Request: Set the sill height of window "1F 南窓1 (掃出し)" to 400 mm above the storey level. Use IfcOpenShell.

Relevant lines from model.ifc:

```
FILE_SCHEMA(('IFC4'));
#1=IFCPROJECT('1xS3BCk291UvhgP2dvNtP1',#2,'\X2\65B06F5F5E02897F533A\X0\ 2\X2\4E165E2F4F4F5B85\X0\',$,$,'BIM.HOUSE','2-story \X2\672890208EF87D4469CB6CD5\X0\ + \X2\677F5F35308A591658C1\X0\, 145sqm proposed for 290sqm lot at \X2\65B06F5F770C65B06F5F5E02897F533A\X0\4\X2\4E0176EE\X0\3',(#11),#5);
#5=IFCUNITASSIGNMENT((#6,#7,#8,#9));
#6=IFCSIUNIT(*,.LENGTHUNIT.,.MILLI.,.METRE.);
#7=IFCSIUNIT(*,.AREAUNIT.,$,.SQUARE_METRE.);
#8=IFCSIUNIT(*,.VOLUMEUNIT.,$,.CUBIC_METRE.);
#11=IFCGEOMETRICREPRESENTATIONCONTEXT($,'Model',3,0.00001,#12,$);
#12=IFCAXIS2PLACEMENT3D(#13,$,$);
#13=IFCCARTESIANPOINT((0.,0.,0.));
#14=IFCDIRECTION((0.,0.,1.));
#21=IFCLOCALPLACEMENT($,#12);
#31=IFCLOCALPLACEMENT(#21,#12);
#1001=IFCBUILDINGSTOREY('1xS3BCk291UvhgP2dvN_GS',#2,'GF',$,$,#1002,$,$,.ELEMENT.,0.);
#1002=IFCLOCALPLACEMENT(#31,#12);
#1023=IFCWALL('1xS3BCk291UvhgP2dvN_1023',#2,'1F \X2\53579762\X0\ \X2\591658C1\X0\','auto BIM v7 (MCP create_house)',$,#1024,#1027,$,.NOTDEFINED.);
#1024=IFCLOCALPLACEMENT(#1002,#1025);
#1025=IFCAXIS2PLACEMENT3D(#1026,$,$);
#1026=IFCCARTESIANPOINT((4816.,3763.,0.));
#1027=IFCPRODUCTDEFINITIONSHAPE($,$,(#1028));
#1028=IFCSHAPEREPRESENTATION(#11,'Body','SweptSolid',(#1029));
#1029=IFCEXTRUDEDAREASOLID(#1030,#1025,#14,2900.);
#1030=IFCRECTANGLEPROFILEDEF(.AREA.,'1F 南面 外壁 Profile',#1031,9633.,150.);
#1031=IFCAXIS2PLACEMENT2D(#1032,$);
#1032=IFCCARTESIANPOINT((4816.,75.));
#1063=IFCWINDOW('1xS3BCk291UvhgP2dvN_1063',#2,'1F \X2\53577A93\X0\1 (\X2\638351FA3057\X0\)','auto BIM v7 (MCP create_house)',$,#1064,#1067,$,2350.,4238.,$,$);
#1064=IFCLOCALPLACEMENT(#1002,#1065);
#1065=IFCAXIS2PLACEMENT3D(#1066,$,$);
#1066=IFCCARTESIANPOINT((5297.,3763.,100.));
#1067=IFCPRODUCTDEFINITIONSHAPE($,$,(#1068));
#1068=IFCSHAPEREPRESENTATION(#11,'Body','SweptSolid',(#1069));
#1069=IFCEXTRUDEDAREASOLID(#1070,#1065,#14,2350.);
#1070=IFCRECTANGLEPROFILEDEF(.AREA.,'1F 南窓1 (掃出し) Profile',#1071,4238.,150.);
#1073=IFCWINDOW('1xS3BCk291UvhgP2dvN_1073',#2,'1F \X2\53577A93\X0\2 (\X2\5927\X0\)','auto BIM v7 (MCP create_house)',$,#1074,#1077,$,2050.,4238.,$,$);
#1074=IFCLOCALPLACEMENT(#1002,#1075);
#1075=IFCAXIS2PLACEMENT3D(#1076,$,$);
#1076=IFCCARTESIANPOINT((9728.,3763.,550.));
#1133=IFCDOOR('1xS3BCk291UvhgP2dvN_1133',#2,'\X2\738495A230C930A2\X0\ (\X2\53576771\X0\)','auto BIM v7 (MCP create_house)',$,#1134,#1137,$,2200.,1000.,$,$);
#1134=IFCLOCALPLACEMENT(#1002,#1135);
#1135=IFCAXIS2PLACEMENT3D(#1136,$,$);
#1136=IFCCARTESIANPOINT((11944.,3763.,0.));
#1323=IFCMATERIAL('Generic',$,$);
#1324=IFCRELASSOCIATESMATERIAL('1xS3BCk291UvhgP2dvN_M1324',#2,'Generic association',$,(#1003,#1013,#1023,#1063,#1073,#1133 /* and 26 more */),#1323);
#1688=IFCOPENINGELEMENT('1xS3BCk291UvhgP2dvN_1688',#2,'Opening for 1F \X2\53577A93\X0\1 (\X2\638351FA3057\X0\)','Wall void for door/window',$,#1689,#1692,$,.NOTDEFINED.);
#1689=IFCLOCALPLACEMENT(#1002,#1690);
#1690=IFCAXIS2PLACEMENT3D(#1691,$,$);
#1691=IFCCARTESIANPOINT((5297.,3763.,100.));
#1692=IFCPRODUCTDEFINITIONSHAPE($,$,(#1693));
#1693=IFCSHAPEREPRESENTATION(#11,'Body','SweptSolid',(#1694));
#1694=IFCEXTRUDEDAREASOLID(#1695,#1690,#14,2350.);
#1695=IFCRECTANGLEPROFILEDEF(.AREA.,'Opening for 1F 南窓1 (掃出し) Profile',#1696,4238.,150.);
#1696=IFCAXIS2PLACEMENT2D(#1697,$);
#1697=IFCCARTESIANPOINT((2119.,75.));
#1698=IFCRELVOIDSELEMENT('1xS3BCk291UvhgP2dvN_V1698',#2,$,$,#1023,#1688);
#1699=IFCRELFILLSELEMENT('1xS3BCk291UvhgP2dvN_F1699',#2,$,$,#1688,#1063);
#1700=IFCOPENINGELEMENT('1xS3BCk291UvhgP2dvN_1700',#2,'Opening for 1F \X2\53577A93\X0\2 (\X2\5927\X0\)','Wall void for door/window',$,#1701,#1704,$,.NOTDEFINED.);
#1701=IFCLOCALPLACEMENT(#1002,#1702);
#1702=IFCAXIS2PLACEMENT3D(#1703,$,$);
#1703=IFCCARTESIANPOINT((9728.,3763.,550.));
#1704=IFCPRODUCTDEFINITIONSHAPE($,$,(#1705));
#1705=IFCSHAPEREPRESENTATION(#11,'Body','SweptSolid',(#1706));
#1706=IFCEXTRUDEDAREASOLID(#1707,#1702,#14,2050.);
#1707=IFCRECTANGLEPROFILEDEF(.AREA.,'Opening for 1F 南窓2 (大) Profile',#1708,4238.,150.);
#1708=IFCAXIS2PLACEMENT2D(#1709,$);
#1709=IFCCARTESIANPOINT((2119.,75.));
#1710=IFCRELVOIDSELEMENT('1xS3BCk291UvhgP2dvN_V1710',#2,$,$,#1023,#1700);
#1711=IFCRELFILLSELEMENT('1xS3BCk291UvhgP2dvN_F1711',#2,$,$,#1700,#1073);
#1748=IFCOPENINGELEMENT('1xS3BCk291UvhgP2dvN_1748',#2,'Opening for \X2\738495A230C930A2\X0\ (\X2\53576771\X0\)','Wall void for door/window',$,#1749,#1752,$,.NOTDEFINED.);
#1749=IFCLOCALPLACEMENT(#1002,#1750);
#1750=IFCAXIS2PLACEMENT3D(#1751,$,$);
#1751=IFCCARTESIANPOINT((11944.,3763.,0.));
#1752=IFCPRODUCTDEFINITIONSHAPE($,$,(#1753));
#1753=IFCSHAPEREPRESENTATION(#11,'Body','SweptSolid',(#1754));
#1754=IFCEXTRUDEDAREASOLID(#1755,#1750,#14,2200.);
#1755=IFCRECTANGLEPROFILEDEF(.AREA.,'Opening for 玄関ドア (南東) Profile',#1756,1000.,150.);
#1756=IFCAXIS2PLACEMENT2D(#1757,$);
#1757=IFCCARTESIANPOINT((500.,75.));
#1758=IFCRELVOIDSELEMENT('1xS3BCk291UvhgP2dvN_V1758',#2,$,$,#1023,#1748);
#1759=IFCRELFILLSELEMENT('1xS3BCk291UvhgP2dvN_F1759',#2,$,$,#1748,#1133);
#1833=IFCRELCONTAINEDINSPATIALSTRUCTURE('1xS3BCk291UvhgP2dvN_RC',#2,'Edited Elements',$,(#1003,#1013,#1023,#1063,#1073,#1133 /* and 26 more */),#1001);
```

```python
import numpy as np
import ifcopenshell
import ifcopenshell.api.geometry
import ifcopenshell.geom
import ifcopenshell.util.element
import ifcopenshell.util.placement
import ifcopenshell.util.shape
import ifcopenshell.util.unit

model = ifcopenshell.open("model.ifc")
unit_scale = ifcopenshell.util.unit.calculate_unit_scale(model)

window = model.by_guid("1xS3BCk291UvhgP2dvN_1063")
opening = window.FillsVoids[0].RelatingOpeningElement
storey = ifcopenshell.util.element.get_container(window, ifc_class="IfcBuildingStorey")
level = ifcopenshell.util.placement.get_local_placement(storey.ObjectPlacement)[2, 3]

# The opening's origin need not be at the sill, so measure its lowest point.
shape = ifcopenshell.geom.create_shape(ifcopenshell.geom.settings(), opening)
bottom = ifcopenshell.util.shape.get_shape_bottom_elevation(shape, shape.geometry) / unit_scale
dz = level + 400.0 - bottom

shift = np.array([0.0, 0.0, dz])
# The window is not placed relative to its opening, so move both.
for product in (opening, window):
    matrix = ifcopenshell.util.placement.get_local_placement(product.ObjectPlacement)
    matrix[:3, 3] += shift
    ifcopenshell.api.geometry.edit_object_placement(model, product=product, matrix=matrix, is_si=False)

print(f"moved by {dz * unit_scale:+.3f} m")

model.write("model_rev.ifc")
```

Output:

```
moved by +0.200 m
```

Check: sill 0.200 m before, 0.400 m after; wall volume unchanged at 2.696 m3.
